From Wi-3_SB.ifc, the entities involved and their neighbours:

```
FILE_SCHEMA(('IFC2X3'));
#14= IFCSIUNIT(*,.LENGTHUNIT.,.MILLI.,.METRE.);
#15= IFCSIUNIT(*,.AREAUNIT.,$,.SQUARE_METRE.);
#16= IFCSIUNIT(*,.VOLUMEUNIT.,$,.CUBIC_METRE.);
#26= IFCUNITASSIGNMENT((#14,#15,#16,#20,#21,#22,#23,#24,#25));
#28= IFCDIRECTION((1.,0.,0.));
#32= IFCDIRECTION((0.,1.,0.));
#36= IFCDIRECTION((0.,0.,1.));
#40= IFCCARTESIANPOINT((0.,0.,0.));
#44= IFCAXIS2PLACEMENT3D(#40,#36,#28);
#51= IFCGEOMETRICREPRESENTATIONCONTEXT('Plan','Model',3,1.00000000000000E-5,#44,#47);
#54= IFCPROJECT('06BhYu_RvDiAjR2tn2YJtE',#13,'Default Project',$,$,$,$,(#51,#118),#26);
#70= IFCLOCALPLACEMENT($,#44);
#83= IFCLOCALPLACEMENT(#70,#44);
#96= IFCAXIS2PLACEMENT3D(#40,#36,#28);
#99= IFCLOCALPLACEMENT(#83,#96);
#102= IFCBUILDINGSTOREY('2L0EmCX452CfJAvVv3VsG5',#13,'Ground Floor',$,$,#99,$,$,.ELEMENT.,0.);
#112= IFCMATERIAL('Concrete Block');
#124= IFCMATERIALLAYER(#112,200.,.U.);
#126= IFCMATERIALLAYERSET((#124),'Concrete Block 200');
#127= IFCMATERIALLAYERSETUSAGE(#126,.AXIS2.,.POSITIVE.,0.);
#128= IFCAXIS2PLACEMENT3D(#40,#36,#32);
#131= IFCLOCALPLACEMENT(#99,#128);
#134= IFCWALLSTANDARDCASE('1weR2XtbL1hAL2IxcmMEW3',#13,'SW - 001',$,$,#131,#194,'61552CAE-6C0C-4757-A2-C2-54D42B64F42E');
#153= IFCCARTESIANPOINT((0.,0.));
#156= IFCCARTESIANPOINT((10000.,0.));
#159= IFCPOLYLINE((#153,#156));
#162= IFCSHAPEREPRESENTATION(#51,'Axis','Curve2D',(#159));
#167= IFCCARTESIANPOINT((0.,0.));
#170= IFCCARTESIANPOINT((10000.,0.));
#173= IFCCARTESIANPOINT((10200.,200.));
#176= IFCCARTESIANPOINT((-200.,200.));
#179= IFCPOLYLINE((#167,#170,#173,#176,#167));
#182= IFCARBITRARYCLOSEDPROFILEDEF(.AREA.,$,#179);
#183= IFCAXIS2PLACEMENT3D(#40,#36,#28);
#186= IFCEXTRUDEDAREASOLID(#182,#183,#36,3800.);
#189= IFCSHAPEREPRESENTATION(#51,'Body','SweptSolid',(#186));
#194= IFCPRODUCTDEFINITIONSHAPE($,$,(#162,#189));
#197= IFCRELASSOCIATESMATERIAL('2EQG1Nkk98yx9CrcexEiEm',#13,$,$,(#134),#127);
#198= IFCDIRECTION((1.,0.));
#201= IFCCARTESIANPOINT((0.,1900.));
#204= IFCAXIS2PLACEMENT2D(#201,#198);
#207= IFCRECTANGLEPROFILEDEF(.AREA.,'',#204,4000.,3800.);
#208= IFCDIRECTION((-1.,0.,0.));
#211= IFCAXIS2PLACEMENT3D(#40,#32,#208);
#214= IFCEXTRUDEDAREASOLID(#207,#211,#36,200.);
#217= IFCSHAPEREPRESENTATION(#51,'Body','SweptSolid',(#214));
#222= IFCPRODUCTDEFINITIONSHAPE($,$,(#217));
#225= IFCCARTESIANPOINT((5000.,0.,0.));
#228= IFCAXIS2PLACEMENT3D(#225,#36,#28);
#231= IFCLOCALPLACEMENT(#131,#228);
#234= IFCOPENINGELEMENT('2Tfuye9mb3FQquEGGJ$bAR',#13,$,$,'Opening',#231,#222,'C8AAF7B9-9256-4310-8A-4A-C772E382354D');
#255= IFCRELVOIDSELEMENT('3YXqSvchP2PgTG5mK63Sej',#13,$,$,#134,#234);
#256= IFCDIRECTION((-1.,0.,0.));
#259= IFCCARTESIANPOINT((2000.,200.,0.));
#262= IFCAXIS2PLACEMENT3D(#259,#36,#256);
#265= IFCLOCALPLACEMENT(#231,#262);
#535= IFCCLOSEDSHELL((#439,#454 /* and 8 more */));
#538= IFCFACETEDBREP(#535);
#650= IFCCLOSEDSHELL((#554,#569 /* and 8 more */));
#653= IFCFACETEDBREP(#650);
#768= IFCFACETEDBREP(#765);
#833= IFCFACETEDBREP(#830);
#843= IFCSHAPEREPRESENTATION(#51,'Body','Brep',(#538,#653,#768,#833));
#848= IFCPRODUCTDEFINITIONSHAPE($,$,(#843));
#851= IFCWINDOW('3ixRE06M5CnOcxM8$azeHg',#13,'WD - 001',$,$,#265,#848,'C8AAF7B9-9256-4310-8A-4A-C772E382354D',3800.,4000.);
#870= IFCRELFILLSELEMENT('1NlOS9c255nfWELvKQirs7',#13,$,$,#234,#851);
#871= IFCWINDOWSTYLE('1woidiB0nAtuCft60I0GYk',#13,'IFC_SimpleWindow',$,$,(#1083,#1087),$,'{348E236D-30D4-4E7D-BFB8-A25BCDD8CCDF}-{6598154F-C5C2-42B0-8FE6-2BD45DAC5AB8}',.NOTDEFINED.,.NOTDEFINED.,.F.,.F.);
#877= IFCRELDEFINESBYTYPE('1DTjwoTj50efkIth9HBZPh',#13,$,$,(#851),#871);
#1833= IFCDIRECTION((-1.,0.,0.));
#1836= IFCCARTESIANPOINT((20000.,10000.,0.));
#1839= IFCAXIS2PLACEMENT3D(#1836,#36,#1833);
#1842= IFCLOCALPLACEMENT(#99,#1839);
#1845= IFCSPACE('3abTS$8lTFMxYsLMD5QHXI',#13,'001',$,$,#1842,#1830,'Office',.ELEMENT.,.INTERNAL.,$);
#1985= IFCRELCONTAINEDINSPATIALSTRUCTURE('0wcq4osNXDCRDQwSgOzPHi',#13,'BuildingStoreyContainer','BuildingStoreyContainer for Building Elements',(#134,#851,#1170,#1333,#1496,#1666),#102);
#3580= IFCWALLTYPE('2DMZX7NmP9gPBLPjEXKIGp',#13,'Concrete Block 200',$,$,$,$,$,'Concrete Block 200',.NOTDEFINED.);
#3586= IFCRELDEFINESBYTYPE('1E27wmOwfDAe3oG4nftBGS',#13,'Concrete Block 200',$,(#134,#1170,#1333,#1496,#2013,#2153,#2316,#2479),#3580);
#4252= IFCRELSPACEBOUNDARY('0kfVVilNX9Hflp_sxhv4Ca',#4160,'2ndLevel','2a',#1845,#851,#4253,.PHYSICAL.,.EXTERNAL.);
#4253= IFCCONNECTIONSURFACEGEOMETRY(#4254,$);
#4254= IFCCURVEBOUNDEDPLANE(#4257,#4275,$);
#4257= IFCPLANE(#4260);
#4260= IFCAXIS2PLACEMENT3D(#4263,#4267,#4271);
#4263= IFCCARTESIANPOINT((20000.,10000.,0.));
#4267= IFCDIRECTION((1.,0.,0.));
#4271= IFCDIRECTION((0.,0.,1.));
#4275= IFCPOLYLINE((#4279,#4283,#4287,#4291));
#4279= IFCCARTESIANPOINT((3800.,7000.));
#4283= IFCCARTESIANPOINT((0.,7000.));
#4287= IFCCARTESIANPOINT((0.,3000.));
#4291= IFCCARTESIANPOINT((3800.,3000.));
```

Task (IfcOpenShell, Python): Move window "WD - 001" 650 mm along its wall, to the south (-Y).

```python
import numpy as np
import ifcopenshell
import ifcopenshell.api.geometry
import ifcopenshell.util.placement

model = ifcopenshell.open("Wi-3_SB.ifc")

window = model.by_guid("3ixRE06M5CnOcxM8$azeHg")
opening = window.FillsVoids[0].RelatingOpeningElement
wall = opening.VoidsElements[0].RelatingBuildingElement

wall_matrix = ifcopenshell.util.placement.get_local_placement(wall.ObjectPlacement)
shift = wall_matrix[:3, 0] * -650.0
before = ifcopenshell.util.placement.get_local_placement(window.ObjectPlacement)[:3, 3].copy()

# The window is placed relative to its opening, so it follows when the opening moves.
matrix = ifcopenshell.util.placement.get_local_placement(opening.ObjectPlacement)
matrix[:3, 3] += shift
ifcopenshell.api.geometry.edit_object_placement(
    model, product=opening, matrix=matrix, is_si=False, should_transform_children=True
)

# Space boundary surfaces are stored in each space's coordinates; move them too.
for rel in window.ProvidesBoundaries:
    if not rel.ConnectionGeometry:
        continue
    surface = rel.ConnectionGeometry.SurfaceOnRelatingElement.BasisSurface
    space_matrix = ifcopenshell.util.placement.get_local_placement(rel.RelatingSpace.ObjectPlacement)
    point = np.array(surface.Position.Location.Coordinates) + space_matrix[:3, :3].T @ shift
    surface.Position = model.createIfcAxis2Placement3D(
        model.createIfcCartesianPoint(point.tolist()), surface.Position.Axis, surface.Position.RefDirection
    )

after = ifcopenshell.util.placement.get_local_placement(window.ObjectPlacement)[:3, 3]
print("window moved by", (after - before).round(3) + 0.0)

model.write("Wi-3_SB_v2.ifc")
```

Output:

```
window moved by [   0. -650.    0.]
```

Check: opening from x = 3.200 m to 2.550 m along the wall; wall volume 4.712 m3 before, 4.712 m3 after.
